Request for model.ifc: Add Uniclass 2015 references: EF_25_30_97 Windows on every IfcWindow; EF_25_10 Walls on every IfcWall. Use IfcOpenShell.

First a look at what the model holds.

```python
import ifcopenshell

model = ifcopenshell.open("model.ifc")
print(model.schema)
print("classifications:", [c.Name for c in model.by_type("IfcClassification")])
for ifc_class in ("IfcDoor", "IfcRoof", "IfcStair", "IfcWall", "IfcWindow"):
    print(ifc_class, len(model.by_type(ifc_class)))
```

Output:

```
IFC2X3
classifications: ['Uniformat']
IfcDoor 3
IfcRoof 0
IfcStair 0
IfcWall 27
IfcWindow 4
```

```python
import ifcopenshell
import ifcopenshell.api.classification

model = ifcopenshell.open("model.ifc")

# IFC2X3 requires Source and Edition and has no link from the project to the system.
system = model.create_entity("IfcClassification", Source="NBS", Edition="2015", Name="Uniclass 2015")

codes = {
    "IfcWindow": ("EF_25_30_97", "Windows"),
    "IfcWall": ("EF_25_10", "Walls"),
}
for ifc_class, (code, name) in codes.items():
    products = model.by_type(ifc_class)
    ifcopenshell.api.classification.add_reference(
        model, products=products, classification=system, identification=code, name=name
    )
    print(code, len(products))

model.write("model_v2.ifc")
```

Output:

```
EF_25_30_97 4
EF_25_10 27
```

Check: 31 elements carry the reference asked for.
